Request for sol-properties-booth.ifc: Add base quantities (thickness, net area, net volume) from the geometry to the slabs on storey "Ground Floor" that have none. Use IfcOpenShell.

First a look at what the model holds.

```python
import ifcopenshell
import ifcopenshell.util.element
import ifcopenshell.util.unit

model = ifcopenshell.open("sol-properties-booth.ifc")
print(model.schema)
for unit_type in ("LENGTHUNIT", "AREAUNIT", "VOLUMEUNIT"):
    print(unit_type, ifcopenshell.util.unit.calculate_unit_scale(model, unit_type))
storey = next(s for s in model.by_type("IfcBuildingStorey") if s.Name == "Ground Floor")
slabs = [e for e in ifcopenshell.util.element.get_decomposition(storey) if e.is_a("IfcSlab")]
for e in sorted(slabs, key=lambda e: e.id()):
    print(e.id(), e.is_a(), e.Name, list(ifcopenshell.util.element.get_psets(e, qtos_only=True)), sep=" | ")
```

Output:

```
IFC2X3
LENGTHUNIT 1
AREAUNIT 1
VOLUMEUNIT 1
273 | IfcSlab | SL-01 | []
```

```python
import ifcopenshell
import ifcopenshell.api.pset
import ifcopenshell.geom
import ifcopenshell.util.element
import ifcopenshell.util.shape
import ifcopenshell.util.unit

model = ifcopenshell.open("sol-properties-booth.ifc")
unit_scale = ifcopenshell.util.unit.calculate_unit_scale(model)
area_scale = ifcopenshell.util.unit.calculate_unit_scale(model, "AREAUNIT")
volume_scale = ifcopenshell.util.unit.calculate_unit_scale(model, "VOLUMEUNIT")
settings = ifcopenshell.geom.settings()

storey = next(s for s in model.by_type("IfcBuildingStorey") if s.Name == "Ground Floor")
slabs = [e for e in ifcopenshell.util.element.get_decomposition(storey) if e.is_a("IfcSlab")]

for e in sorted(slabs, key=lambda e: e.id()):
    if ifcopenshell.util.element.get_psets(e, qtos_only=True, should_inherit=False):
        continue
    # Geometry comes back in metres, in the element's own axes.
    shape = ifcopenshell.geom.create_shape(settings, e)
    values = {
        "Width": ifcopenshell.util.shape.get_z(shape.geometry) / unit_scale,
        "NetArea": ifcopenshell.util.shape.get_footprint_area(shape.geometry) / area_scale,
        "NetVolume": ifcopenshell.util.shape.get_volume(shape.geometry) / volume_scale,
    }
    qto = ifcopenshell.api.pset.add_qto(model, product=e, name="BaseQuantities")
    ifcopenshell.api.pset.edit_qto(model, qto=qto, properties=values)
    print(e.id(), {k: round(v, 3) for k, v in values.items()})

model.write("sol-properties-booth-out.ifc")
```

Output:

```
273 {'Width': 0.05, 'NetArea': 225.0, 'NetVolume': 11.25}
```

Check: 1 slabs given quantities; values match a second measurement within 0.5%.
